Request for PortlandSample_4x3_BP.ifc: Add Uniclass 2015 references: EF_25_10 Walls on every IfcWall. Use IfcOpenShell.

First a look at what the model holds.

```python
import ifcopenshell

model = ifcopenshell.open("PortlandSample_4x3_BP.ifc")
print(model.schema)
print("classifications:", [c.Name for c in model.by_type("IfcClassification")])
for ifc_class in ("IfcDoor", "IfcRoof", "IfcStair", "IfcWall", "IfcWindow"):
    print(ifc_class, len(model.by_type(ifc_class)))
```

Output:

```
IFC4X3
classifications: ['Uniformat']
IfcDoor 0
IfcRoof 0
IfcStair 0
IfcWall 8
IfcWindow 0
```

```python
import ifcopenshell
import ifcopenshell.api.classification

model = ifcopenshell.open("PortlandSample_4x3_BP.ifc")

system = ifcopenshell.api.classification.add_classification(model, classification="Uniclass 2015")

codes = {
    "IfcWall": ("EF_25_10", "Walls"),
}
for ifc_class, (code, name) in codes.items():
    products = model.by_type(ifc_class)
    ifcopenshell.api.classification.add_reference(
        model, products=products, classification=system, identification=code, name=name
    )
    print(code, len(products))

model.write("PortlandSample_4x3_BP_v2.ifc")
```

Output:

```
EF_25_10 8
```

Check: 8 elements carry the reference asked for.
